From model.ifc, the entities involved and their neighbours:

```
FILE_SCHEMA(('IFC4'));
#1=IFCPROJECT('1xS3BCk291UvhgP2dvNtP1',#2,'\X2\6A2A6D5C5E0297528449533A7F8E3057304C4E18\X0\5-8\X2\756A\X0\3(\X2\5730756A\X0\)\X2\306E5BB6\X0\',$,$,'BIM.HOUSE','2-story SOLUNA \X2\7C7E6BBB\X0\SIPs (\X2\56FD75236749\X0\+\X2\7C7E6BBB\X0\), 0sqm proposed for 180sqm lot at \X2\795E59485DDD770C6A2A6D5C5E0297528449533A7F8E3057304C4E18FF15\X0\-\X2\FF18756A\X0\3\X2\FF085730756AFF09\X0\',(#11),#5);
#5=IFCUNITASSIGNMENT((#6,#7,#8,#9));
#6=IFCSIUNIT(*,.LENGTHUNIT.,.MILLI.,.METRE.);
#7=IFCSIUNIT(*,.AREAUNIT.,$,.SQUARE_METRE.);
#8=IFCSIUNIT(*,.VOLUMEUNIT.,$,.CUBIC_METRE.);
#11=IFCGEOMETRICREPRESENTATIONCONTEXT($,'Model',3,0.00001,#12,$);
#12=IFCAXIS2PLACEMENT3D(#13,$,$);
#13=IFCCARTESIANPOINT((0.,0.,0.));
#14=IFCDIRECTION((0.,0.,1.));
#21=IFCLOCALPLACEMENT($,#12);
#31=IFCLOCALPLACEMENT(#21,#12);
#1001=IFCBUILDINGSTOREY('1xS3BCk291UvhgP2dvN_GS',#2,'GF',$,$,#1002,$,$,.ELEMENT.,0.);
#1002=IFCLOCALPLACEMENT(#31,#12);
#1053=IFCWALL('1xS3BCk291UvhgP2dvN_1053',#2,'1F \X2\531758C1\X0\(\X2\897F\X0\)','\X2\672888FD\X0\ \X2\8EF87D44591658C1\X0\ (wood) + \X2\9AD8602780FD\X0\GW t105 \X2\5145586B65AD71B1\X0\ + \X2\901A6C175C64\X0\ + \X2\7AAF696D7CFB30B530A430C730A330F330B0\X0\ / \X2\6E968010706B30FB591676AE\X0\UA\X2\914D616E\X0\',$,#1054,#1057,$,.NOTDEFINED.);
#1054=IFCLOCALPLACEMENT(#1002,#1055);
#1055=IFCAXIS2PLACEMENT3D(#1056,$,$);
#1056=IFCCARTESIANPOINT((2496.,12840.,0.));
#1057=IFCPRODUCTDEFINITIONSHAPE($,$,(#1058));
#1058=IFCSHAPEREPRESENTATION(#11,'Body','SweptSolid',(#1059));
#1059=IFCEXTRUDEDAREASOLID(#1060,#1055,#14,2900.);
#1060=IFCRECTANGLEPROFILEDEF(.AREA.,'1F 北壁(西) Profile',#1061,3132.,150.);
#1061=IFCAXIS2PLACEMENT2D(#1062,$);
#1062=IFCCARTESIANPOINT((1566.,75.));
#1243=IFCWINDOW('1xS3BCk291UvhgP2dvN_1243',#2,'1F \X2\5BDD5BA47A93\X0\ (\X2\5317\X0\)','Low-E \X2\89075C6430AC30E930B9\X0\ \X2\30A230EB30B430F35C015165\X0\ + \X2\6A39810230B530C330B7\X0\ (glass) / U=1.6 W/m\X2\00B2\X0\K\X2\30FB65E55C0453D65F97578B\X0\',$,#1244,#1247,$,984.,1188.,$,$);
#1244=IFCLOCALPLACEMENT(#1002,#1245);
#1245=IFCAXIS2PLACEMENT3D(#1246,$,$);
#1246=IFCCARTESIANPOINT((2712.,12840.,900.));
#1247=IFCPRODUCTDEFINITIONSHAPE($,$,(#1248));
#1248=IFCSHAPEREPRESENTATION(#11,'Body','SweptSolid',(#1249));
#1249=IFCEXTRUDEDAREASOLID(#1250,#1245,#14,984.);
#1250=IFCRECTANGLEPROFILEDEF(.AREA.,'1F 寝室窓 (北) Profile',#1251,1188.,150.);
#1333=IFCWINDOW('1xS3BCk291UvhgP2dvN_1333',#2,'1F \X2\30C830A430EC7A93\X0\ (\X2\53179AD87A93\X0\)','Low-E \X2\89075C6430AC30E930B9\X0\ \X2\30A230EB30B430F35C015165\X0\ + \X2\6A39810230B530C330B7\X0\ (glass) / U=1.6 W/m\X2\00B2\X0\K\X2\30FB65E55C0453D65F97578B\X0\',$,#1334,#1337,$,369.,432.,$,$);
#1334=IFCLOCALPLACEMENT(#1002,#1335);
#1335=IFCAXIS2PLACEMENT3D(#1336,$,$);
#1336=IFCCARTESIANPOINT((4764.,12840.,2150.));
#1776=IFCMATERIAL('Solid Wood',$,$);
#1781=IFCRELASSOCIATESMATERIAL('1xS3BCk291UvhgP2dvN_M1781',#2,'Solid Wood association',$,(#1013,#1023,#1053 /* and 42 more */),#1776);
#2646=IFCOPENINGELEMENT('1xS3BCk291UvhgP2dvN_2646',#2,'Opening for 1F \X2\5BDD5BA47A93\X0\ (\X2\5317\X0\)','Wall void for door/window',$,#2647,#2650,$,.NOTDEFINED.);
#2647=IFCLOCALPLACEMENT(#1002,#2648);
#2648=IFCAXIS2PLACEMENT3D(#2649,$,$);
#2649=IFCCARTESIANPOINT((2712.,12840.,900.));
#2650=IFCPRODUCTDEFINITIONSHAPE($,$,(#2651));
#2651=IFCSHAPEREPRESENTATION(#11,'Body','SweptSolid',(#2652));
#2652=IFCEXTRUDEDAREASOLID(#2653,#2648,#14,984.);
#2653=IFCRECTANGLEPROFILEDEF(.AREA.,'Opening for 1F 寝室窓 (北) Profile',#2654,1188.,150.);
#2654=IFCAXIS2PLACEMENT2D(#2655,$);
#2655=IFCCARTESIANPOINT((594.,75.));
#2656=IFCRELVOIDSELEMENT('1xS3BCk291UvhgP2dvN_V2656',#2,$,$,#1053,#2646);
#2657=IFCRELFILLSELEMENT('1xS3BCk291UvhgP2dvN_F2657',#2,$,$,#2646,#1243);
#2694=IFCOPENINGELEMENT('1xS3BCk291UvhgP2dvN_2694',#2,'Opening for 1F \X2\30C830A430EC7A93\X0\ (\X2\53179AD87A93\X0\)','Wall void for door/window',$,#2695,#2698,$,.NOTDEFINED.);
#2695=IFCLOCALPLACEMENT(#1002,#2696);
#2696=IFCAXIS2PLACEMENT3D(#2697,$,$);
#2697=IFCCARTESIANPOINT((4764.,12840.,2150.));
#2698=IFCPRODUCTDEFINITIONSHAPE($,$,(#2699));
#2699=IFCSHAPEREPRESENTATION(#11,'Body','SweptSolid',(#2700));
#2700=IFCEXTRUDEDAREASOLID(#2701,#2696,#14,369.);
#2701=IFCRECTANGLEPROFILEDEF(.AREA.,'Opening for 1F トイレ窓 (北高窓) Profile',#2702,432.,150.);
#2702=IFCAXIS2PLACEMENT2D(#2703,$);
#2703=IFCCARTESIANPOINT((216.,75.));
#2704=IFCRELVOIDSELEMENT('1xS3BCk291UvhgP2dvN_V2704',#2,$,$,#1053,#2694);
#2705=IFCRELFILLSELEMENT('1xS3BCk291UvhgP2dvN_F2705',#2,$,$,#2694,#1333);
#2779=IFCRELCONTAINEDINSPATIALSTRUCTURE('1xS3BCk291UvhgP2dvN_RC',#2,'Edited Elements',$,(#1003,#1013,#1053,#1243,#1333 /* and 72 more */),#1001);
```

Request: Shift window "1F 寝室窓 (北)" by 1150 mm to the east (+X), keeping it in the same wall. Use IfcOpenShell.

```python
import ifcopenshell
import ifcopenshell.api.geometry
import ifcopenshell.util.placement

model = ifcopenshell.open("model.ifc")

window = model.by_guid("1xS3BCk291UvhgP2dvN_1243")
opening = window.FillsVoids[0].RelatingOpeningElement
wall = opening.VoidsElements[0].RelatingBuildingElement

wall_matrix = ifcopenshell.util.placement.get_local_placement(wall.ObjectPlacement)
shift = wall_matrix[:3, 0] * 1150.0
before = ifcopenshell.util.placement.get_local_placement(window.ObjectPlacement)[:3, 3].copy()

# The window is not placed relative to its opening, so move both.
for product in (opening, window):
    matrix = ifcopenshell.util.placement.get_local_placement(product.ObjectPlacement)
    matrix[:3, 3] += shift
    ifcopenshell.api.geometry.edit_object_placement(model, product=product, matrix=matrix, is_si=False)

after = ifcopenshell.util.placement.get_local_placement(window.ObjectPlacement)[:3, 3]
print("window moved by", (after - before).round(3) + 0.0)

model.write("model-out.ifc")
```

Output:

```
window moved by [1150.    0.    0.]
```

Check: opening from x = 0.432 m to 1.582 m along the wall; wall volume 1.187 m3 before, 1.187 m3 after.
